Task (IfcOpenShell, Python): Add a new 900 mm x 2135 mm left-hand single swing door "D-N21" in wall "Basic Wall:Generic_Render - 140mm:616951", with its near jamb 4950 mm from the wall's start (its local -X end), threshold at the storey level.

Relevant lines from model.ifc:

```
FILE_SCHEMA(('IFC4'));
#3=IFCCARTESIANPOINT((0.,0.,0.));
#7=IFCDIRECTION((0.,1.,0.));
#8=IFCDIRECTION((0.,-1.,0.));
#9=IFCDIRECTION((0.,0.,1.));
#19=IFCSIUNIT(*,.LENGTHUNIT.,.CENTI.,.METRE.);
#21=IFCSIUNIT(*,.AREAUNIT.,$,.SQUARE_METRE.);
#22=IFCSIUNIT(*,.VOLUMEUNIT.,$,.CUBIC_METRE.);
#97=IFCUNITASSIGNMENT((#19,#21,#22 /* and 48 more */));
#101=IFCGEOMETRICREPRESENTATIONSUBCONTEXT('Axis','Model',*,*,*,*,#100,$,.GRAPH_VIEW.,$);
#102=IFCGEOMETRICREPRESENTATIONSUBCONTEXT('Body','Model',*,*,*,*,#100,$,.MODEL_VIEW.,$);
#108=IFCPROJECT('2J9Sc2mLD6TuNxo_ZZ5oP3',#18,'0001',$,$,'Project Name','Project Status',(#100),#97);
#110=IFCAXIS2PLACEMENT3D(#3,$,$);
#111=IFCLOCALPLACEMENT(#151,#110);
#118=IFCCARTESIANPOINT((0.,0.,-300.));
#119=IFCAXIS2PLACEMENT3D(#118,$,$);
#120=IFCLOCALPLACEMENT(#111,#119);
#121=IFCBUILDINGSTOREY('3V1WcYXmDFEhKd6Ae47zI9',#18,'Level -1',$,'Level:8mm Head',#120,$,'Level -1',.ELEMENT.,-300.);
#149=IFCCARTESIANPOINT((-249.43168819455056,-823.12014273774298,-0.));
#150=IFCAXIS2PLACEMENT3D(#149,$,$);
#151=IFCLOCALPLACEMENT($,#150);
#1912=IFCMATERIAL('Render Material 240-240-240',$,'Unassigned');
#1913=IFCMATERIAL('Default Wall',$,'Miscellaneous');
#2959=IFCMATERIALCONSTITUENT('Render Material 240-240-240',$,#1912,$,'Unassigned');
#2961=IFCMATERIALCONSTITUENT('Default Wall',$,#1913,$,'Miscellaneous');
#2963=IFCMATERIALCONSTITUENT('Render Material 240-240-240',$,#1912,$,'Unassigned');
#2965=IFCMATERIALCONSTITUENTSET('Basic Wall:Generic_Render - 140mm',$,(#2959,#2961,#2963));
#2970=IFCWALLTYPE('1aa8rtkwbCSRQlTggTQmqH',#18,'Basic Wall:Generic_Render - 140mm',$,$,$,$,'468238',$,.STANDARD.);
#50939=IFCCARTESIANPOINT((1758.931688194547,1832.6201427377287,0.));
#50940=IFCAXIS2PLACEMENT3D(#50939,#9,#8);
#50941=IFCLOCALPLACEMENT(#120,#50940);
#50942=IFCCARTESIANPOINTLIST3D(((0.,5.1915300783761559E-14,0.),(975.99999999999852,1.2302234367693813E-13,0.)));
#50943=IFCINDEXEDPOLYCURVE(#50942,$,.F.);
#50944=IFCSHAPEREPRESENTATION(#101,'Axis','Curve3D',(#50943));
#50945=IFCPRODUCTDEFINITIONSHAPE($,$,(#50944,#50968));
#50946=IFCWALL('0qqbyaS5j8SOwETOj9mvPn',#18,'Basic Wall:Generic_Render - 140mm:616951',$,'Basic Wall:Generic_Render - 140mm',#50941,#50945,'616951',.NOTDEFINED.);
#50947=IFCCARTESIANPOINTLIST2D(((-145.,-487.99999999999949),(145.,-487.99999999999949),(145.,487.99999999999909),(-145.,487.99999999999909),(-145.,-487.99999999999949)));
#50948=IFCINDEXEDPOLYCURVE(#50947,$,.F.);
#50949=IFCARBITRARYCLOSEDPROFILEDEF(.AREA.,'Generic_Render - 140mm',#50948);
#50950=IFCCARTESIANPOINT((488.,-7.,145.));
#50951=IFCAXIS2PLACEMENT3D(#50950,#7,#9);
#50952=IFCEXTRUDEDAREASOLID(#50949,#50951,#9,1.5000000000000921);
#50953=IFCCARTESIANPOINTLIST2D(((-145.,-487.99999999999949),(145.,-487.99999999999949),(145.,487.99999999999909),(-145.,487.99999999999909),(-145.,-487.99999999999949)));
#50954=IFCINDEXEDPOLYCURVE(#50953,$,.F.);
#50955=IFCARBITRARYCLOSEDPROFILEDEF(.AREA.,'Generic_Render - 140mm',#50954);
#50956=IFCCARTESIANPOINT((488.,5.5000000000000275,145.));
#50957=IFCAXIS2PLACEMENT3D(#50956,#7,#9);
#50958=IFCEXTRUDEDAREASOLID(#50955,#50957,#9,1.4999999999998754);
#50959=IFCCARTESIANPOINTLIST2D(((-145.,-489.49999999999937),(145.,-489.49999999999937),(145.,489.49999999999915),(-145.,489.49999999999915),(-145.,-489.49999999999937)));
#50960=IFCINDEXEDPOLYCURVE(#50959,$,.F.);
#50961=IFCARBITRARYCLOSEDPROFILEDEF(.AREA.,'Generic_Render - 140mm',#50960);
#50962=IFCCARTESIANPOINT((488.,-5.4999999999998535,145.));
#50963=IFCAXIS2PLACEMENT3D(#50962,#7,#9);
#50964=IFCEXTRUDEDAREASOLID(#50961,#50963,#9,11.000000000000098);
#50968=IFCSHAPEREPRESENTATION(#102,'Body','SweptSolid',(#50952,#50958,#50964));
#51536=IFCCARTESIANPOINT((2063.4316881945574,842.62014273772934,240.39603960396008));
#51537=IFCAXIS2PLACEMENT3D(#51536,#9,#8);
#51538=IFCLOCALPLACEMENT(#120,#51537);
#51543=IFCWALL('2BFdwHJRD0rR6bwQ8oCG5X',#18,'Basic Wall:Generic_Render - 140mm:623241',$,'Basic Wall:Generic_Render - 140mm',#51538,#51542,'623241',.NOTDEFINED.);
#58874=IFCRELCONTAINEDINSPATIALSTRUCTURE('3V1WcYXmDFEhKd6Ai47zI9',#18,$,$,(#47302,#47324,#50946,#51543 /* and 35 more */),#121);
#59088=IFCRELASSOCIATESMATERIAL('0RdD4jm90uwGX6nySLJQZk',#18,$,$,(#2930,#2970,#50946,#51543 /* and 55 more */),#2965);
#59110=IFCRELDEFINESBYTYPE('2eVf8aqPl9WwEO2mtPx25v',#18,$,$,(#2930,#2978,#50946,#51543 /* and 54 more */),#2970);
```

```python
import numpy as np
import ifcopenshell
import ifcopenshell.api.feature
import ifcopenshell.api.geometry
import ifcopenshell.api.root
import ifcopenshell.api.spatial
import ifcopenshell.geom
import ifcopenshell.util.element
import ifcopenshell.util.placement
import ifcopenshell.util.representation
import ifcopenshell.util.shape
import ifcopenshell.util.unit

model = ifcopenshell.open("model.ifc")
unit_scale = ifcopenshell.util.unit.calculate_unit_scale(model)
settings = ifcopenshell.geom.settings()


def volume(element):
    """Net volume in cubic metres, openings subtracted."""
    shape = ifcopenshell.geom.create_shape(settings, element)
    return ifcopenshell.util.shape.get_volume(shape.geometry)


wall = model.by_id(50946)
storey = ifcopenshell.util.element.get_container(wall, ifc_class="IfcBuildingStorey")
context = ifcopenshell.util.representation.get_context(model, "Model", "Body", "MODEL_VIEW")
before = volume(wall)

width, height, from_end, sill = 0.9, 2.135, 4.95, 0.0  # metres

# The wall runs along its own X axis, and the end named is its -X end.
wall_shape = ifcopenshell.geom.create_shape(settings, wall)
x, y, z = ifcopenshell.util.shape.get_vertices(wall_shape.geometry).T
start = x.min() + from_end
face, thickness = float(y.min()), float(y.max() - y.min())
wall_matrix = ifcopenshell.util.placement.get_local_placement(wall.ObjectPlacement)
level = ifcopenshell.util.placement.get_local_placement(storey.ObjectPlacement)[2, 3]


def in_wall(x, y):
    """Placement at x, y metres in the wall's axes, at sill height."""
    matrix = wall_matrix.copy()
    matrix[:, 3] = wall_matrix @ np.array([x / unit_scale, y / unit_scale, 0.0, 1.0])
    matrix[2, 3] = level + sill / unit_scale
    return matrix


# Opening: a box that overshoots both wall faces by 50 mm.
opening = ifcopenshell.api.root.create_entity(model, ifc_class="IfcOpeningElement", predefined_type="OPENING")
box = ifcopenshell.api.geometry.add_wall_representation(
    model, context=context, length=width, height=height, thickness=thickness + 0.1
)
ifcopenshell.api.geometry.assign_representation(model, product=opening, representation=box)
ifcopenshell.api.geometry.edit_object_placement(model, product=opening, matrix=in_wall(start, face - 0.05), is_si=False)
ifcopenshell.api.feature.add_feature(model, feature=opening, element=wall)

door = ifcopenshell.api.root.create_entity(model, ifc_class="IfcDoor", name="D-N21", predefined_type="DOOR")
door.OverallWidth, door.OverallHeight = width / unit_scale, height / unit_scale
door.OperationType = "SINGLE_SWING_LEFT"
body = ifcopenshell.api.geometry.add_door_representation(
    model,
    context=context,
    overall_width=door.OverallWidth,
    overall_height=door.OverallHeight,
    operation_type="SINGLE_SWING_LEFT",
    lining_properties={"LiningDepth": thickness / unit_scale, "ThresholdDepth": thickness / unit_scale},
)
ifcopenshell.api.geometry.assign_representation(model, product=door, representation=body)
ifcopenshell.api.spatial.assign_container(model, products=[door], relating_structure=storey)
ifcopenshell.api.feature.add_filling(model, opening=opening, element=door)

# The lining spans the wall, so the door starts at the wall face.
ifcopenshell.api.geometry.edit_object_placement(model, product=door, matrix=in_wall(start, face), is_si=False)

after = volume(wall)

print(f"wall volume {before:.3f} -> {after:.3f} m3")

model.write("model_v2.ifc")
```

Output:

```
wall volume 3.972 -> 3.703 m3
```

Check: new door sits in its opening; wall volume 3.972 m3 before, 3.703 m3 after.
